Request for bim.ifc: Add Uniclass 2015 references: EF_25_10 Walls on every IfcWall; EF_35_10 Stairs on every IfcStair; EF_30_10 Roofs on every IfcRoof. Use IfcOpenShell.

First a look at what the model holds.

```python
import ifcopenshell

model = ifcopenshell.open("bim.ifc")
print(model.schema)
print("classifications:", [c.Name for c in model.by_type("IfcClassification")])
for ifc_class in ("IfcDoor", "IfcRoof", "IfcStair", "IfcWall", "IfcWindow"):
    print(ifc_class, len(model.by_type(ifc_class)))
```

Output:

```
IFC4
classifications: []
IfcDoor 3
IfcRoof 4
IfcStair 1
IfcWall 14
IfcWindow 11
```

```python
import ifcopenshell
import ifcopenshell.api.classification

model = ifcopenshell.open("bim.ifc")

system = ifcopenshell.api.classification.add_classification(model, classification="Uniclass 2015")

codes = {
    "IfcWall": ("EF_25_10", "Walls"),
    "IfcStair": ("EF_35_10", "Stairs"),
    "IfcRoof": ("EF_30_10", "Roofs"),
}
for ifc_class, (code, name) in codes.items():
    products = model.by_type(ifc_class)
    ifcopenshell.api.classification.add_reference(
        model, products=products, classification=system, identification=code, name=name
    )
    print(code, len(products))

model.write("bim_v2.ifc")
```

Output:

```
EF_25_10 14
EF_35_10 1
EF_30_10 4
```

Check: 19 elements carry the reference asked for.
